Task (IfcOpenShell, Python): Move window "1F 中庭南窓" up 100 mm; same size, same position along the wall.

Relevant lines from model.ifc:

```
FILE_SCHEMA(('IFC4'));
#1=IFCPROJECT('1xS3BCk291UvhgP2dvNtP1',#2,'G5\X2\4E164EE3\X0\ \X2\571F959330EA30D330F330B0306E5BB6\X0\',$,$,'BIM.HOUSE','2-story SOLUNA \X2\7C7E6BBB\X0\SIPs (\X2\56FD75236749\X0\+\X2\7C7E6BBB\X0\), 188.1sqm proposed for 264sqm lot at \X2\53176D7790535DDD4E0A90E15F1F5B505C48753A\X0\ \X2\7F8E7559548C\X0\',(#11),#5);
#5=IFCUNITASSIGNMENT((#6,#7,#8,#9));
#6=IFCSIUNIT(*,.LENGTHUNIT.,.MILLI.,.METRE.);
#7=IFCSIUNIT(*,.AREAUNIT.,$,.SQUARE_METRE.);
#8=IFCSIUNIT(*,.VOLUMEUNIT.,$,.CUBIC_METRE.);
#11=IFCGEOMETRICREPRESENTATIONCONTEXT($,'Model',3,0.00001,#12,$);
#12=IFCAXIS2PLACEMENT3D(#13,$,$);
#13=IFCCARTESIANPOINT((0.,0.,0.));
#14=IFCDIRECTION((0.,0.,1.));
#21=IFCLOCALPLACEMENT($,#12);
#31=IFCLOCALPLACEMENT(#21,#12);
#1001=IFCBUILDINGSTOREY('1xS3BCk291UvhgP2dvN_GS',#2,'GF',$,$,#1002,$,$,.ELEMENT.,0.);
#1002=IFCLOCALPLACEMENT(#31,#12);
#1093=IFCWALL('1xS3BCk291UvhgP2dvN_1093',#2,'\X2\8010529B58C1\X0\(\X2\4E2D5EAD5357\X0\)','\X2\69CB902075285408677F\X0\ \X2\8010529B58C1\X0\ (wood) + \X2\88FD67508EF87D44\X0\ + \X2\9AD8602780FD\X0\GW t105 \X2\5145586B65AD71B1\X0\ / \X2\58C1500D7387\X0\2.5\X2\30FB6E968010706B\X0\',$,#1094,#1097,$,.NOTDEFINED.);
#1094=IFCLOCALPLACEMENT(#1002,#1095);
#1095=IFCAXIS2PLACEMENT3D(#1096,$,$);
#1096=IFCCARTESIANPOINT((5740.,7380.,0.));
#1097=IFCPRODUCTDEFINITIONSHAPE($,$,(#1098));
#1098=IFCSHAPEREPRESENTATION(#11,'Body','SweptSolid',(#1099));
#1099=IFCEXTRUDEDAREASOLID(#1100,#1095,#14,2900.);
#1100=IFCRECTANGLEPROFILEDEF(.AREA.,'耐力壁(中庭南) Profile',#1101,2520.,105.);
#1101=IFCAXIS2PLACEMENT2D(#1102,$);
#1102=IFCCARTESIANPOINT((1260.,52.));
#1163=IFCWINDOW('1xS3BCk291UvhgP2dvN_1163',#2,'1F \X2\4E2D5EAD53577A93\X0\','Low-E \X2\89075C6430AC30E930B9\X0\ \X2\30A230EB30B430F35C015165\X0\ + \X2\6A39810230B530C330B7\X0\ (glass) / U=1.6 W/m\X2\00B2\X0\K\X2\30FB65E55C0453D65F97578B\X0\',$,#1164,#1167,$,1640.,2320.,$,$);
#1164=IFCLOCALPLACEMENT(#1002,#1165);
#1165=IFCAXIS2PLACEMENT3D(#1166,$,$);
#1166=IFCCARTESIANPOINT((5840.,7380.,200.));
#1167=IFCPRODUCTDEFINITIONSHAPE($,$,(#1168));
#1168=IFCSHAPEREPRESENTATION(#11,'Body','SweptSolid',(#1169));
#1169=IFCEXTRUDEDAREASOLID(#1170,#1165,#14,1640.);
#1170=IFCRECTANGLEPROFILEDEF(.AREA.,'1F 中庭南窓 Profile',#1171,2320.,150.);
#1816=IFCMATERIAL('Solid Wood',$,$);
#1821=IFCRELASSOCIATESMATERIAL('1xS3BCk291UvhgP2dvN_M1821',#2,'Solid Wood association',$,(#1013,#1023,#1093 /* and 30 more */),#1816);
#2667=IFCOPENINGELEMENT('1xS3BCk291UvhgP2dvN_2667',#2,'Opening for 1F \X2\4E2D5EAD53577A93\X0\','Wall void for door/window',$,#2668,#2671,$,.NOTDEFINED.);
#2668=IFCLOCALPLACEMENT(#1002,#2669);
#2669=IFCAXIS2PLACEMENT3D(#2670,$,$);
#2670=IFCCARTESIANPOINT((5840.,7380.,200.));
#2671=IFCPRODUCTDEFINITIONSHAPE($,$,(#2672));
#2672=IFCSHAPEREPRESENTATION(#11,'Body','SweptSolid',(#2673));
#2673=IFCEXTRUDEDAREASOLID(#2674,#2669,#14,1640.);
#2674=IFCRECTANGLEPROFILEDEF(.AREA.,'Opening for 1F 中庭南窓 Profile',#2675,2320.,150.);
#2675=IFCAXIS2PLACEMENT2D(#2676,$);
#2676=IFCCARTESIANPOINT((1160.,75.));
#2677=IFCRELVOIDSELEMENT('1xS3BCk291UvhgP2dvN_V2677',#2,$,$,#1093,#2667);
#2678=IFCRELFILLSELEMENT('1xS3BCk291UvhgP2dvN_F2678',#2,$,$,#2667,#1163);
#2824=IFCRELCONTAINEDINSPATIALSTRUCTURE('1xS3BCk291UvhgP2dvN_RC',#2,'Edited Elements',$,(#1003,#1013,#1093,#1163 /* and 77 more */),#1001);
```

```python
import numpy as np
import ifcopenshell
import ifcopenshell.api.geometry
import ifcopenshell.util.placement
import ifcopenshell.util.unit

model = ifcopenshell.open("model.ifc")
unit_scale = ifcopenshell.util.unit.calculate_unit_scale(model)

window = model.by_guid("1xS3BCk291UvhgP2dvN_1163")
opening = window.FillsVoids[0].RelatingOpeningElement
dz = 0.1 / unit_scale

shift = np.array([0.0, 0.0, dz])
# The window is not placed relative to its opening, so move both.
for product in (opening, window):
    matrix = ifcopenshell.util.placement.get_local_placement(product.ObjectPlacement)
    matrix[:3, 3] += shift
    ifcopenshell.api.geometry.edit_object_placement(model, product=product, matrix=matrix, is_si=False)

print(f"moved by {dz * unit_scale:+.3f} m")

model.write("model_updated.ifc")
```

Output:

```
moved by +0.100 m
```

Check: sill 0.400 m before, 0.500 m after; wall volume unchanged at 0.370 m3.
